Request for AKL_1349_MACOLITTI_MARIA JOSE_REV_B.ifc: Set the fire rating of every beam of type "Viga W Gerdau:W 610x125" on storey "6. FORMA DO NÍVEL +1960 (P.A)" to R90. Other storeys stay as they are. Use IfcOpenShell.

First a look at what the model holds.

```python
import ifcopenshell
import ifcopenshell.util.element

model = ifcopenshell.open("AKL_1349_MACOLITTI_MARIA JOSE_REV_B.ifc")
print(model.schema)
storey = next(s for s in model.by_type("IfcBuildingStorey") if s.Name == "6. FORMA DO NÍVEL +1960 (P.A)")
beams = [e for e in ifcopenshell.util.element.get_decomposition(storey) if e.is_a("IfcBeam")]
seen = {}
for e in beams:
    element_type = ifcopenshell.util.element.get_type(e)
    key = (element_type.Name if element_type != e and element_type else None, ifcopenshell.util.element.get_pset(e, "Pset_BeamCommon", "FireRating"))
    seen[key] = seen.get(key, 0) + 1
for (name, value), count in sorted(seen.items(), key=str):
    print(count, "x", name, "|", value)
```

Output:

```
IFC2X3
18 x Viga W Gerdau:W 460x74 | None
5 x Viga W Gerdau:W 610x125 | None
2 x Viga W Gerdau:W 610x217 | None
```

```python
import ifcopenshell
import ifcopenshell.api.pset
import ifcopenshell.util.element

model = ifcopenshell.open("AKL_1349_MACOLITTI_MARIA JOSE_REV_B.ifc")

storey = next(s for s in model.by_type("IfcBuildingStorey") if s.Name == "6. FORMA DO NÍVEL +1960 (P.A)")
beams = [e for e in ifcopenshell.util.element.get_decomposition(storey) if e.is_a("IfcBeam")]

count = 0
for e in beams:
    element_type = ifcopenshell.util.element.get_type(e)
    if element_type in (None, e) or element_type.Name != "Viga W Gerdau:W 610x125":
        continue
    # add_pset returns the element's existing set when there is one.
    pset = ifcopenshell.api.pset.add_pset(model, product=e, name="Pset_BeamCommon")
    ifcopenshell.api.pset.edit_pset(model, pset=pset, properties={"FireRating": "R90"})
    count += 1

print(count, "beams updated")

model.write("AKL_1349_MACOLITTI_MARIA JOSE_REV_B_v2.ifc")
```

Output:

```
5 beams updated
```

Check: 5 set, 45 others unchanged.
